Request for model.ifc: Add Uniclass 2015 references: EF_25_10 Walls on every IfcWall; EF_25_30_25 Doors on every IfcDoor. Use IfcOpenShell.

First a look at what the model holds.

```python
import ifcopenshell

model = ifcopenshell.open("model.ifc")
print(model.schema)
print("classifications:", [c.Name for c in model.by_type("IfcClassification")])
for ifc_class in ("IfcDoor", "IfcRoof", "IfcStair", "IfcWall", "IfcWindow"):
    print(ifc_class, len(model.by_type(ifc_class)))
```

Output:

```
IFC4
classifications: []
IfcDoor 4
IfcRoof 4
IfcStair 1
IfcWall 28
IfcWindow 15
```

```python
import ifcopenshell
import ifcopenshell.api.classification

model = ifcopenshell.open("model.ifc")

system = ifcopenshell.api.classification.add_classification(model, classification="Uniclass 2015")

codes = {
    "IfcWall": ("EF_25_10", "Walls"),
    "IfcDoor": ("EF_25_30_25", "Doors"),
}
for ifc_class, (code, name) in codes.items():
    products = model.by_type(ifc_class)
    ifcopenshell.api.classification.add_reference(
        model, products=products, classification=system, identification=code, name=name
    )
    print(code, len(products))

model.write("model-out.ifc")
```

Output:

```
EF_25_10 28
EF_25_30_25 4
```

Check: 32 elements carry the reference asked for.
